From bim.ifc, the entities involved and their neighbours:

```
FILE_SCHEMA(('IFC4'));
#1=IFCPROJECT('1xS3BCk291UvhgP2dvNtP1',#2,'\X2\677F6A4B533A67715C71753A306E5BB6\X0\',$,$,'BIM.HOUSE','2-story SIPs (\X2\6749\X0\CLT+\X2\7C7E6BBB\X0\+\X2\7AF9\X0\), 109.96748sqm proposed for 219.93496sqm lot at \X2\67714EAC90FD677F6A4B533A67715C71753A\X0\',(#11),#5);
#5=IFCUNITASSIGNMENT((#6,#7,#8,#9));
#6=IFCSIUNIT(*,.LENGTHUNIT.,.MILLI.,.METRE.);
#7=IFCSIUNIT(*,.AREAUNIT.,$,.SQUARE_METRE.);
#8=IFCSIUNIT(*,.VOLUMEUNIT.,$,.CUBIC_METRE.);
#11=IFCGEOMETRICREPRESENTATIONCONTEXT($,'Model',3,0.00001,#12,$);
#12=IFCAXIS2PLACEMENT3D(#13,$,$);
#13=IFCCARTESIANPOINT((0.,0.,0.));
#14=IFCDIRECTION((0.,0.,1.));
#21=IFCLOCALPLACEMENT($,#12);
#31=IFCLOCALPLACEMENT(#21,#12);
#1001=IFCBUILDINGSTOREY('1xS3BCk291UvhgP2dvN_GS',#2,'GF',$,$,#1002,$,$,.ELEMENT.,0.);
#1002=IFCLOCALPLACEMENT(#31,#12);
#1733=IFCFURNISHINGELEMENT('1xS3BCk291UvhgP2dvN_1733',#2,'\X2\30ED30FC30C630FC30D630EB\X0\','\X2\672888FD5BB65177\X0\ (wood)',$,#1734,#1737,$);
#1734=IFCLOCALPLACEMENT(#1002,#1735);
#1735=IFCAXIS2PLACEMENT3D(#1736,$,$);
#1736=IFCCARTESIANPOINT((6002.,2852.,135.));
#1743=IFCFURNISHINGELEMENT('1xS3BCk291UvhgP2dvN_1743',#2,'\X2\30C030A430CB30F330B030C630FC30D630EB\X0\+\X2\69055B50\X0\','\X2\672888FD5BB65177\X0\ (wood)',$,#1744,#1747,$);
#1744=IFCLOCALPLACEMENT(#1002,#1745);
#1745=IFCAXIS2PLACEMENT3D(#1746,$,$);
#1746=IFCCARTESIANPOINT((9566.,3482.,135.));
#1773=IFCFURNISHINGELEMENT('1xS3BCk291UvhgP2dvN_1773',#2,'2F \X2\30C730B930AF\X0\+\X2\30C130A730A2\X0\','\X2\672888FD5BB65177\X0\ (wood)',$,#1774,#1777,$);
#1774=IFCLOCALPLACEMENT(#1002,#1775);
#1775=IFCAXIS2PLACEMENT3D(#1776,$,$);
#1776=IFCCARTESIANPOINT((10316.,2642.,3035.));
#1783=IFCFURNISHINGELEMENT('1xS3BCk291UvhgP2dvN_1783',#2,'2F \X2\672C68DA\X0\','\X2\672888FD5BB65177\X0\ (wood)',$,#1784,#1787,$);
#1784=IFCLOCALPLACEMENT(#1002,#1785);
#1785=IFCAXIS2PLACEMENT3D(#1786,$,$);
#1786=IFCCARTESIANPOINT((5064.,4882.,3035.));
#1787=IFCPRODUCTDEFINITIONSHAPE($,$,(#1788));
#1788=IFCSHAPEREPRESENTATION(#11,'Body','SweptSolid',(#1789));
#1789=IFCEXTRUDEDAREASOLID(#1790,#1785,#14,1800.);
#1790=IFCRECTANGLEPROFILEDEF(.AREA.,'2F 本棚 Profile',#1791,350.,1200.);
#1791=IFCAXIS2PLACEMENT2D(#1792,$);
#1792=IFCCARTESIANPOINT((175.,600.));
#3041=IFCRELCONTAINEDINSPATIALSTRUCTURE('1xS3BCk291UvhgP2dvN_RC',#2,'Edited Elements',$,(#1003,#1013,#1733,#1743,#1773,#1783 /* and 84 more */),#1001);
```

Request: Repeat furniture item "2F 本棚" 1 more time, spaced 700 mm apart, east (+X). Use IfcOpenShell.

```python
import numpy as np
import ifcopenshell
import ifcopenshell.api.geometry
import ifcopenshell.api.root
import ifcopenshell.util.element
import ifcopenshell.util.placement

model = ifcopenshell.open("bim.ifc")


def reuse_history(source, copy):
    """copy_class also copies each property set's owner history, people and application; keep the originals."""
    for rel in copy.IsDefinedBy:
        if rel.is_a("IfcRelDefinesByProperties") and (history := rel.RelatingPropertyDefinition.OwnerHistory):
            rel.RelatingPropertyDefinition.OwnerHistory = source.OwnerHistory
            ifcopenshell.util.element.remove_deep2(model, history)


source = model.by_id(1783)
base = ifcopenshell.util.placement.get_local_placement(source.ObjectPlacement)
step = np.array([1.0, 0.0, 0.0]) * 700.0

for i in range(1, 2):
    copy = ifcopenshell.api.root.copy_class(model, product=source)
    copy.Representation = ifcopenshell.util.element.copy_deep(
        model, source.Representation, exclude=["IfcGeometricRepresentationContext", "IfcRepresentationMap"]
    )
    reuse_history(source, copy)
    matrix = base.copy()
    matrix[:3, 3] += i * step
    print("added at", matrix[:3, 3].round(3) + 0.0)
    ifcopenshell.api.geometry.edit_object_placement(model, product=copy, matrix=matrix, is_si=False)

model.write("bim-out.ifc")
```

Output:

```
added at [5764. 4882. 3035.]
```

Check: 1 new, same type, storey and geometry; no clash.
